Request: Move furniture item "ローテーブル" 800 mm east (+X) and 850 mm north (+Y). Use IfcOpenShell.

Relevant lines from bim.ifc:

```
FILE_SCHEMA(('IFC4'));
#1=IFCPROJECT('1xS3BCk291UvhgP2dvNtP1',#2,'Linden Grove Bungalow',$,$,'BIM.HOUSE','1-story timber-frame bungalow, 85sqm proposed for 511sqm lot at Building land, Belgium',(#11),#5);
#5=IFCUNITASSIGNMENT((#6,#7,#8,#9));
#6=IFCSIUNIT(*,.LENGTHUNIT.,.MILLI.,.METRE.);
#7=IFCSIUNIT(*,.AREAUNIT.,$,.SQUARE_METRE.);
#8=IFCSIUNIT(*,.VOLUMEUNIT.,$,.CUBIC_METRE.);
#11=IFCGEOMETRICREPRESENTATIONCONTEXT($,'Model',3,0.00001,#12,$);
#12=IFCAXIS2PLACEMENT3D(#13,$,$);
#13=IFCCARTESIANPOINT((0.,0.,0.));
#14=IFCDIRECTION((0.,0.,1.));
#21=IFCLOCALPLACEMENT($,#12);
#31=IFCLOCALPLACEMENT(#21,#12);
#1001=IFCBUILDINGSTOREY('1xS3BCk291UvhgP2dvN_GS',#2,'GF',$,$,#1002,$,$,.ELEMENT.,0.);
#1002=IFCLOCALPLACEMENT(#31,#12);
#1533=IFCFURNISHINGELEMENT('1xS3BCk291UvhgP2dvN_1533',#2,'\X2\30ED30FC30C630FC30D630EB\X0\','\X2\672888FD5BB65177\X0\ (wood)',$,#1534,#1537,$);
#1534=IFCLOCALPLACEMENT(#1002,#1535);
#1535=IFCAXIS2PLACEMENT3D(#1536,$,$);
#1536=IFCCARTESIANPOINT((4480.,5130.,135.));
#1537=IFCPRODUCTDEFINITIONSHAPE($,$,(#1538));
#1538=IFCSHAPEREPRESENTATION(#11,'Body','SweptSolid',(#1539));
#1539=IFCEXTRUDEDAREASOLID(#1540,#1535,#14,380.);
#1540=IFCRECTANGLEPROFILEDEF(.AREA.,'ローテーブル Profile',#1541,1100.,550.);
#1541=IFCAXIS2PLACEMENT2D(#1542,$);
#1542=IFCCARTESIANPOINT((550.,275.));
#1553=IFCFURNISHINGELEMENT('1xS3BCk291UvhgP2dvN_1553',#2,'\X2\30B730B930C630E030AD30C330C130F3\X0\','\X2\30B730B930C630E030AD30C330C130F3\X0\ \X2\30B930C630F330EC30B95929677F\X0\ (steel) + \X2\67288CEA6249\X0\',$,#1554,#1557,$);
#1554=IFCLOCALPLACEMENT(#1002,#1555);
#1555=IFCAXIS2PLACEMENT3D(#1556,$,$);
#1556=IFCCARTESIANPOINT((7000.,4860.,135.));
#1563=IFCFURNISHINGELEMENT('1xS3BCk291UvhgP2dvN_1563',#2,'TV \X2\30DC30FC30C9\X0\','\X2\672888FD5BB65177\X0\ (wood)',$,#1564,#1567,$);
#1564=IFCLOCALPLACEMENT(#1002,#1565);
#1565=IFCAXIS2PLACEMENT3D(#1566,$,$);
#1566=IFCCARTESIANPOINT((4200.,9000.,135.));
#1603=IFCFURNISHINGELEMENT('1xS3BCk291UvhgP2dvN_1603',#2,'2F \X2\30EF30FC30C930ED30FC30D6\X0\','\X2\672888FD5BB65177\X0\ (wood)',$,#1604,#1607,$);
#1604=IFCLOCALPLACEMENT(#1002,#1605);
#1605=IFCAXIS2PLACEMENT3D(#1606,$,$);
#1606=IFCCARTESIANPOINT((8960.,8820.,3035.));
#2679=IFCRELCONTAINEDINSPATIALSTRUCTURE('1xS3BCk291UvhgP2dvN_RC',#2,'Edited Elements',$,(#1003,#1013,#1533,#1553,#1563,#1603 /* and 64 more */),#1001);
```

```python
import ifcopenshell
import ifcopenshell.api.geometry
import ifcopenshell.util.placement
import ifcopenshell.util.unit

model = ifcopenshell.open("bim.ifc")
unit_scale = ifcopenshell.util.unit.calculate_unit_scale(model)

item = model.by_id(1533)
matrix = ifcopenshell.util.placement.get_local_placement(item.ObjectPlacement)
matrix[0, 3] += 0.8 / unit_scale
matrix[1, 3] += 0.85 / unit_scale
ifcopenshell.api.geometry.edit_object_placement(model, product=item, matrix=matrix, is_si=False)

print(ifcopenshell.util.placement.get_local_placement(item.ObjectPlacement).round(3) + 0.0)

model.write("bim_updated.ifc")
```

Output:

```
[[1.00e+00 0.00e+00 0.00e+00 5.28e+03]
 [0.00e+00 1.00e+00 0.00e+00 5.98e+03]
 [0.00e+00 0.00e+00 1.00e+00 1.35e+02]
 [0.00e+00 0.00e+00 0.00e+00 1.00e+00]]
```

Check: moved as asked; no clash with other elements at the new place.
